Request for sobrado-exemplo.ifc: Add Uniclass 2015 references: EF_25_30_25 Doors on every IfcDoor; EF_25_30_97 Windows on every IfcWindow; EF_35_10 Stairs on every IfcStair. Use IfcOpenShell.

First a look at what the model holds.

```python
import ifcopenshell

model = ifcopenshell.open("sobrado-exemplo.ifc")
print(model.schema)
print("classifications:", [c.Name for c in model.by_type("IfcClassification")])
for ifc_class in ("IfcDoor", "IfcRoof", "IfcStair", "IfcWall", "IfcWindow"):
    print(ifc_class, len(model.by_type(ifc_class)))
```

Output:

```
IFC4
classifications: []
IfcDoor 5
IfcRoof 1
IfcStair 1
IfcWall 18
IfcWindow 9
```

```python
import ifcopenshell
import ifcopenshell.api.classification

model = ifcopenshell.open("sobrado-exemplo.ifc")

system = ifcopenshell.api.classification.add_classification(model, classification="Uniclass 2015")

codes = {
    "IfcDoor": ("EF_25_30_25", "Doors"),
    "IfcWindow": ("EF_25_30_97", "Windows"),
    "IfcStair": ("EF_35_10", "Stairs"),
}
for ifc_class, (code, name) in codes.items():
    products = model.by_type(ifc_class)
    ifcopenshell.api.classification.add_reference(
        model, products=products, classification=system, identification=code, name=name
    )
    print(code, len(products))

model.write("sobrado-exemplo_v2.ifc")
```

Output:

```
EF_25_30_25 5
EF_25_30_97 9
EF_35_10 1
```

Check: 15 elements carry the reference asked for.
